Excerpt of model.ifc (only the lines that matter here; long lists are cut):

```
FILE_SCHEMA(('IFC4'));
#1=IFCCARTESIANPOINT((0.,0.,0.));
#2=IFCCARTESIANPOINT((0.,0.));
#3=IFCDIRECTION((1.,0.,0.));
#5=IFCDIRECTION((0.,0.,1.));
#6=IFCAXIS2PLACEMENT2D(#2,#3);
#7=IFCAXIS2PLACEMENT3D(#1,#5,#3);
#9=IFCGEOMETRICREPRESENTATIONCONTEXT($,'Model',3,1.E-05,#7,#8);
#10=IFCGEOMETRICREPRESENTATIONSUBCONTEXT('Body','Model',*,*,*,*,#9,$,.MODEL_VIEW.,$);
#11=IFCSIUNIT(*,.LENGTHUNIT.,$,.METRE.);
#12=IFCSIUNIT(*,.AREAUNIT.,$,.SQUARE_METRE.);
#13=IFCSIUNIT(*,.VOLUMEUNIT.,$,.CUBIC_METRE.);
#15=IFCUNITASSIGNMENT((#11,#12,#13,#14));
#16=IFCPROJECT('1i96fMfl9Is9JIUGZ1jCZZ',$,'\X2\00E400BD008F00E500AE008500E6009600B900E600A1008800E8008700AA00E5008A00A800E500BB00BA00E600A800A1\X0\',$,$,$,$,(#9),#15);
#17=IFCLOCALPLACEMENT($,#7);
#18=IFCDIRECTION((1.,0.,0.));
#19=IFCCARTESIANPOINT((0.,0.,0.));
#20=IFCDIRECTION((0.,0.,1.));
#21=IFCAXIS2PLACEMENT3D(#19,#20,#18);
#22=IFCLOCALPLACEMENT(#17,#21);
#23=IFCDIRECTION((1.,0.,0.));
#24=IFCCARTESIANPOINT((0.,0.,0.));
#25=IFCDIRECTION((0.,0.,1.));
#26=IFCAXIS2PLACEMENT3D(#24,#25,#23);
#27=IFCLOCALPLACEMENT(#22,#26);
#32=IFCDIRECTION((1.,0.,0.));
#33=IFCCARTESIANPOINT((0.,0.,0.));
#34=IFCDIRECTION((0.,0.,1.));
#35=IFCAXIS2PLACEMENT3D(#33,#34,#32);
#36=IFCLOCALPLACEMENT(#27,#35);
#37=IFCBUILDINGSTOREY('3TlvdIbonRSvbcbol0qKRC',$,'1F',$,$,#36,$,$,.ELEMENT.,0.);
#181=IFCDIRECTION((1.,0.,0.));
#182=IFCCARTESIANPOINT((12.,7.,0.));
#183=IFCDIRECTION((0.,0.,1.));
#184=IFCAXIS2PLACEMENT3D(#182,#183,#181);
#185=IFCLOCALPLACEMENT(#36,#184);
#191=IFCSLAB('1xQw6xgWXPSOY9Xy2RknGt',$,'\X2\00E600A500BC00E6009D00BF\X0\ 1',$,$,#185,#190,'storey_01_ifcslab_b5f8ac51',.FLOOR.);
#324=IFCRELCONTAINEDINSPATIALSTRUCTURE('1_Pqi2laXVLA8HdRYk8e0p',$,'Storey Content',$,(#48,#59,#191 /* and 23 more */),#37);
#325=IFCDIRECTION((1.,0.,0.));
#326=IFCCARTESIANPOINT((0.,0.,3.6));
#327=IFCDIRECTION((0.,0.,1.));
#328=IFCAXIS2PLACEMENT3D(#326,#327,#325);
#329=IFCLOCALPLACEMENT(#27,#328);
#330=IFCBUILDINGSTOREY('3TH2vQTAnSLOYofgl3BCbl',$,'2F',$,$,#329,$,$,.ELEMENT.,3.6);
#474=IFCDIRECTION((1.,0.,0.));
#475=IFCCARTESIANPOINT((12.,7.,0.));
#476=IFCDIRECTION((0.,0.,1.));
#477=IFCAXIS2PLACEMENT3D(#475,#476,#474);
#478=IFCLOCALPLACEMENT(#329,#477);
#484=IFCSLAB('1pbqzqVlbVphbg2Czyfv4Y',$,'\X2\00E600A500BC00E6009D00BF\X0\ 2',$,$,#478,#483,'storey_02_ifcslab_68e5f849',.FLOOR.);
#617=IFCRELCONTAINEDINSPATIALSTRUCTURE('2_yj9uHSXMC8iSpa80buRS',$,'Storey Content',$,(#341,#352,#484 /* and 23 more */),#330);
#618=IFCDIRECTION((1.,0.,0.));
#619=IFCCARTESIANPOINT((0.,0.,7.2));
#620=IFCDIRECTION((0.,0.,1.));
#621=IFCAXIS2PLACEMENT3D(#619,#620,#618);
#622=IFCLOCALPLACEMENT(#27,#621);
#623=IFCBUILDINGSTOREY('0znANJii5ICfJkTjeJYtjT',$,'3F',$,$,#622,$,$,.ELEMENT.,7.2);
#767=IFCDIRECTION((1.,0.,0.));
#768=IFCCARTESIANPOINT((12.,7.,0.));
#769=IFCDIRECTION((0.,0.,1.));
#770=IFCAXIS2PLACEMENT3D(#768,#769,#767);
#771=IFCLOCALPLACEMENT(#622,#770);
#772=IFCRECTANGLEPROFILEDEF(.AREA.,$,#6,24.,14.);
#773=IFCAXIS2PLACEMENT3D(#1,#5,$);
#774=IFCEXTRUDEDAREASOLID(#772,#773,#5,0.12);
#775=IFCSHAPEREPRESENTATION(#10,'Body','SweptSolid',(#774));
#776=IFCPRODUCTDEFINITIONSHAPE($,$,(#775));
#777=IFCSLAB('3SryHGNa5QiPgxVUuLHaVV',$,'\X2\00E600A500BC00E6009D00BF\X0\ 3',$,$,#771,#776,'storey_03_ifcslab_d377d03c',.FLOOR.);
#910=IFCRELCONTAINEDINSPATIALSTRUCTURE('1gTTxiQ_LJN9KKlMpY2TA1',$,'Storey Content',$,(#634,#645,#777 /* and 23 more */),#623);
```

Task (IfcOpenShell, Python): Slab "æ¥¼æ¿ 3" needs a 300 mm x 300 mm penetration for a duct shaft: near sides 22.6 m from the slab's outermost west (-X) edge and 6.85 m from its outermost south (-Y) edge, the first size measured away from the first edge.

```python
import numpy as np
import ifcopenshell
import ifcopenshell.api.feature
import ifcopenshell.api.geometry
import ifcopenshell.api.root
import ifcopenshell.geom
import ifcopenshell.util.placement
import ifcopenshell.util.representation
import ifcopenshell.util.shape
import ifcopenshell.util.unit

model = ifcopenshell.open("model.ifc")
unit_scale = ifcopenshell.util.unit.calculate_unit_scale(model)
settings = ifcopenshell.geom.settings()


def volume(element):
    """Net volume in cubic metres, openings subtracted."""
    shape = ifcopenshell.geom.create_shape(settings, element)
    return ifcopenshell.util.shape.get_volume(shape.geometry)


slab = model.by_guid("3SryHGNa5QiPgxVUuLHaVV")
before = volume(slab)

# Extent in the slab's own axes, in metres. The edges named are its -X and -Y sides.
slab_shape = ifcopenshell.geom.create_shape(settings, slab)
vertices = ifcopenshell.util.shape.get_vertices(slab_shape.geometry)
x_min, y_min, bottom = vertices.min(axis=0)
top = vertices[:, 2].max()

opening = ifcopenshell.api.root.create_entity(model, ifc_class="IfcOpeningElement", name="Duct shaft opening", predefined_type="OPENING")
context = ifcopenshell.util.representation.get_context(model, "Model", "Body", "MODEL_VIEW")
width, depth = 0.3, 0.3
outline = [(0.0, 0.0), (width, 0.0), (width, depth), (0.0, depth), (0.0, 0.0)]
# Overshoot both faces by 50 mm so the cut is clean.
shape = ifcopenshell.api.geometry.add_slab_representation(
    model, context=context, depth=top - bottom + 0.1, polyline=outline
)
ifcopenshell.api.geometry.assign_representation(model, product=opening, representation=shape)

matrix = ifcopenshell.util.placement.get_local_placement(slab.ObjectPlacement)
matrix[:, 3] = matrix @ np.append(np.array([x_min + 22.6, y_min + 6.85, bottom - 0.05]) / unit_scale, 1.0)
ifcopenshell.api.geometry.edit_object_placement(model, product=opening, matrix=matrix, is_si=False)
ifcopenshell.api.feature.add_feature(model, feature=opening, element=slab)

after = volume(slab)

print(f"slab volume {before:.3f} -> {after:.3f} m3")

model.write("model_edited.ifc")
```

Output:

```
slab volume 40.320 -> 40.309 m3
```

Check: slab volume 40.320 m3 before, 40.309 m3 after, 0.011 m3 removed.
